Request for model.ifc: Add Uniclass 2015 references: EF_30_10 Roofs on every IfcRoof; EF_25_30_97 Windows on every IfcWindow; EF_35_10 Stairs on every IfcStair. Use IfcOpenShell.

First a look at what the model holds.

```python
import ifcopenshell

model = ifcopenshell.open("model.ifc")
print(model.schema)
print("classifications:", [c.Name for c in model.by_type("IfcClassification")])
for ifc_class in ("IfcDoor", "IfcRoof", "IfcStair", "IfcWall", "IfcWindow"):
    print(ifc_class, len(model.by_type(ifc_class)))
```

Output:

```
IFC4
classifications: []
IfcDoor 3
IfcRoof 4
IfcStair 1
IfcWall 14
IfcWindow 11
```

```python
import ifcopenshell
import ifcopenshell.api.classification

model = ifcopenshell.open("model.ifc")

system = ifcopenshell.api.classification.add_classification(model, classification="Uniclass 2015")

codes = {
    "IfcRoof": ("EF_30_10", "Roofs"),
    "IfcWindow": ("EF_25_30_97", "Windows"),
    "IfcStair": ("EF_35_10", "Stairs"),
}
for ifc_class, (code, name) in codes.items():
    products = model.by_type(ifc_class)
    ifcopenshell.api.classification.add_reference(
        model, products=products, classification=system, identification=code, name=name
    )
    print(code, len(products))

model.write("model_updated.ifc")
```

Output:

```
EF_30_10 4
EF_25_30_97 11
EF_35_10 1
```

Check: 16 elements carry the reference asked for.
